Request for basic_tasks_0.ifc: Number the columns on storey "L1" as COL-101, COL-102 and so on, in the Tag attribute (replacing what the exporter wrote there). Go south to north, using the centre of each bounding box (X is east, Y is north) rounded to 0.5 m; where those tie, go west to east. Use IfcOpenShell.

First a look at what the model holds.

```python
import ifcopenshell
import ifcopenshell.util.element
import ifcopenshell.util.placement

model = ifcopenshell.open("basic_tasks_0.ifc")
print(model.schema)
storey = next(s for s in model.by_type("IfcBuildingStorey") if s.Name == "L1")
columns = [e for e in ifcopenshell.util.element.get_decomposition(storey) if e.is_a("IfcColumn")]
for e in sorted(columns, key=lambda e: e.id()):
    origin = ifcopenshell.util.placement.get_local_placement(e.ObjectPlacement)[:3, 3]
    print(e.id(), e.Tag, e.Name, origin.round(2) + 0.0, sep=" | ")
```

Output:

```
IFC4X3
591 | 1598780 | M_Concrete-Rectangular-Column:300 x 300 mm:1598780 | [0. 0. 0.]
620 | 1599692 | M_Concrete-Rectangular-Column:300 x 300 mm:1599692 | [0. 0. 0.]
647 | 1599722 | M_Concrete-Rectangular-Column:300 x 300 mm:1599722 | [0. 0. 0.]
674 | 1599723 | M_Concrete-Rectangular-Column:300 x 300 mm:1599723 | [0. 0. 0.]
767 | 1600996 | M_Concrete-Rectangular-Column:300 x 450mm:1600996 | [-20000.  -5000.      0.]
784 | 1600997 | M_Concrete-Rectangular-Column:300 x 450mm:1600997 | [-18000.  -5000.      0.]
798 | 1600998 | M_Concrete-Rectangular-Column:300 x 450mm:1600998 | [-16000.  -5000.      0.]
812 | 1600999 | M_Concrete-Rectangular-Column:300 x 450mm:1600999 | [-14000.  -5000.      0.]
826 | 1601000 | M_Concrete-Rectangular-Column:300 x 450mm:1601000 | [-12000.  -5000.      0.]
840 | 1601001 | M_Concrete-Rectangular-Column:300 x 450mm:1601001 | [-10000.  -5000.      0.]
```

```python
import ifcopenshell
import ifcopenshell.geom
import ifcopenshell.util.element
import ifcopenshell.util.shape

model = ifcopenshell.open("basic_tasks_0.ifc")
settings = ifcopenshell.geom.settings()
settings.set("use-world-coords", True)


def centre(element):
    shape = ifcopenshell.geom.create_shape(settings, element)
    return ifcopenshell.util.shape.get_bbox_centroid(shape.geometry)


storey = next(s for s in model.by_type("IfcBuildingStorey") if s.Name == "L1")
columns = [e for e in ifcopenshell.util.element.get_decomposition(storey) if e.is_a("IfcColumn")]

# Insertion points can sit at a corner or the storey origin, so sort by the geometry (in metres).
centres = {e: centre(e) for e in columns}
columns.sort(key=lambda e: (round(centres[e][1] / 0.5), centres[e][0]))

for i, e in enumerate(columns, start=1):
    number = f"COL-1{i:02d}"
    e.Tag = number
    print(e.id(), number)

model.write("basic_tasks_0_updated.ifc")
```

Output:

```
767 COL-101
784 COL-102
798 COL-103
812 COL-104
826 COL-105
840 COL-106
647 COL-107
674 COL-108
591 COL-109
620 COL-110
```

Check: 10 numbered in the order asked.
